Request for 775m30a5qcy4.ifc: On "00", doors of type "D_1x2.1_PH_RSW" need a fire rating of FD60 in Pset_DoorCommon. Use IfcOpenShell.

First a look at what the model holds.

```python
import ifcopenshell
import ifcopenshell.util.element

model = ifcopenshell.open("775m30a5qcy4.ifc")
print(model.schema)
storey = next(s for s in model.by_type("IfcBuildingStorey") if s.Name == "00")
doors = [e for e in ifcopenshell.util.element.get_decomposition(storey) if e.is_a("IfcDoor")]
seen = {}
for e in doors:
    element_type = ifcopenshell.util.element.get_type(e)
    key = (element_type.Name if element_type != e and element_type else None, ifcopenshell.util.element.get_pset(e, "Pset_DoorCommon", "FireRating"))
    seen[key] = seen.get(key, 0) + 1
for (name, value), count in sorted(seen.items(), key=str):
    print(count, "x", name, "|", value)
```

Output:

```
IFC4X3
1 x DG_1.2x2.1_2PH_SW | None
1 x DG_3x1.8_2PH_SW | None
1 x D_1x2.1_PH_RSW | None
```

```python
import ifcopenshell
import ifcopenshell.api.pset
import ifcopenshell.util.element

model = ifcopenshell.open("775m30a5qcy4.ifc")

storey = next(s for s in model.by_type("IfcBuildingStorey") if s.Name == "00")
doors = [e for e in ifcopenshell.util.element.get_decomposition(storey) if e.is_a("IfcDoor")]

count = 0
for e in doors:
    element_type = ifcopenshell.util.element.get_type(e)
    if element_type in (None, e) or element_type.Name != "D_1x2.1_PH_RSW":
        continue
    # add_pset returns the element's existing set when there is one.
    pset = ifcopenshell.api.pset.add_pset(model, product=e, name="Pset_DoorCommon")
    ifcopenshell.api.pset.edit_pset(model, pset=pset, properties={"FireRating": "FD60"})
    count += 1

print(count, "doors updated")

model.write("775m30a5qcy4_edited.ifc")
```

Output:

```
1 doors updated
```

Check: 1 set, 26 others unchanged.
